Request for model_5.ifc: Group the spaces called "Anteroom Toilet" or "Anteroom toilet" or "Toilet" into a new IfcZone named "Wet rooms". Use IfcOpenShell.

First a look at what the model holds.

```python
import ifcopenshell

model = ifcopenshell.open("model_5.ifc")
print(model.schema)
seen = {}
for space in model.by_type("IfcSpace"):
    seen[space.LongName] = seen.get(space.LongName, 0) + 1
for name, count in sorted(seen.items(), key=str):
    print(count, "x", name)
print("zones:", [z.Name for z in model.by_type("IfcZone")][:20])
```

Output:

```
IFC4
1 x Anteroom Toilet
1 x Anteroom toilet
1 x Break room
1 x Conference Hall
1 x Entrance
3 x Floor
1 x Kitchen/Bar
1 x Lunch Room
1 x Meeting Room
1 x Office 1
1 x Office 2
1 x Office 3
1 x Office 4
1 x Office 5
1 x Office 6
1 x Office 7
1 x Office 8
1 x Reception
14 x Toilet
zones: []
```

```python
import ifcopenshell
import ifcopenshell.api.group
import ifcopenshell.api.root

model = ifcopenshell.open("model_5.ifc")

names = {"Anteroom Toilet", "Anteroom toilet", "Toilet"}
spaces = [s for s in model.by_type("IfcSpace") if s.LongName in names]

zone = ifcopenshell.api.root.create_entity(model, ifc_class="IfcZone", name="Wet rooms")
ifcopenshell.api.group.assign_group(model, products=spaces, group=zone)
print(len(spaces), "spaces in", zone.Name)

model.write("model_5_updated.ifc")
```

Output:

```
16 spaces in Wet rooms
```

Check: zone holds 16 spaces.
